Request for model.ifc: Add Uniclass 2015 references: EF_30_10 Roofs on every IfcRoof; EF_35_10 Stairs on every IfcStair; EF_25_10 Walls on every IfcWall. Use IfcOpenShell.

First a look at what the model holds.

```python
import ifcopenshell

model = ifcopenshell.open("model.ifc")
print(model.schema)
print("classifications:", [c.Name for c in model.by_type("IfcClassification")])
for ifc_class in ("IfcDoor", "IfcRoof", "IfcStair", "IfcWall", "IfcWindow"):
    print(ifc_class, len(model.by_type(ifc_class)))
```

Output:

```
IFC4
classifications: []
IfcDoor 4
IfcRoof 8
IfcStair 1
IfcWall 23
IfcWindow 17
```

```python
import ifcopenshell
import ifcopenshell.api.classification

model = ifcopenshell.open("model.ifc")

system = ifcopenshell.api.classification.add_classification(model, classification="Uniclass 2015")

codes = {
    "IfcRoof": ("EF_30_10", "Roofs"),
    "IfcStair": ("EF_35_10", "Stairs"),
    "IfcWall": ("EF_25_10", "Walls"),
}
for ifc_class, (code, name) in codes.items():
    products = model.by_type(ifc_class)
    ifcopenshell.api.classification.add_reference(
        model, products=products, classification=system, identification=code, name=name
    )
    print(code, len(products))

model.write("model_v2.ifc")
```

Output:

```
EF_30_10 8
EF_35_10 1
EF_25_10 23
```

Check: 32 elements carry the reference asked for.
